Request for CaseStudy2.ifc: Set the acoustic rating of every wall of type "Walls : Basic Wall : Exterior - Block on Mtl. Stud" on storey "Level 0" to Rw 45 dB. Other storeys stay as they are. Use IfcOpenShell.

First a look at what the model holds.

```python
import ifcopenshell
import ifcopenshell.util.element

model = ifcopenshell.open("CaseStudy2.ifc")
print(model.schema)
storey = next(s for s in model.by_type("IfcBuildingStorey") if s.Name == "Level 0")
walls = [e for e in ifcopenshell.util.element.get_decomposition(storey) if e.is_a("IfcWall")]
seen = {}
for e in walls:
    element_type = ifcopenshell.util.element.get_type(e)
    key = (element_type.Name if element_type != e and element_type else None, ifcopenshell.util.element.get_pset(e, "Pset_WallCommon", "AcousticRating"))
    seen[key] = seen.get(key, 0) + 1
for (name, value), count in sorted(seen.items(), key=str):
    print(count, "x", name, "|", value)
```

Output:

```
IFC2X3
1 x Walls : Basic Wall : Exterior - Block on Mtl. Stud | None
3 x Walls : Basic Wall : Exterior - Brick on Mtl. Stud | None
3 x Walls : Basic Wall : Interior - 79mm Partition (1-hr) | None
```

```python
import ifcopenshell
import ifcopenshell.api.pset
import ifcopenshell.util.element

model = ifcopenshell.open("CaseStudy2.ifc")

storey = next(s for s in model.by_type("IfcBuildingStorey") if s.Name == "Level 0")
walls = [e for e in ifcopenshell.util.element.get_decomposition(storey) if e.is_a("IfcWall")]

count = 0
for e in walls:
    element_type = ifcopenshell.util.element.get_type(e)
    if element_type in (None, e) or element_type.Name != "Walls : Basic Wall : Exterior - Block on Mtl. Stud":
        continue
    # add_pset returns the element's existing set when there is one.
    pset = ifcopenshell.api.pset.add_pset(model, product=e, name="Pset_WallCommon")
    ifcopenshell.api.pset.edit_pset(model, pset=pset, properties={"AcousticRating": "Rw 45 dB"})
    count += 1

print(count, "walls updated")

model.write("CaseStudy2_updated.ifc")
```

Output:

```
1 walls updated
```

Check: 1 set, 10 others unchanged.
